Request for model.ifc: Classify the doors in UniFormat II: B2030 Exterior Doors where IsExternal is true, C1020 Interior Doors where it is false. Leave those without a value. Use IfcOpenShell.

First a look at what the model holds.

```python
import ifcopenshell
import ifcopenshell.util.element

model = ifcopenshell.open("model.ifc")
print(model.schema)
print("classifications:", [c.Name for c in model.by_type("IfcClassification")])
values = [ifcopenshell.util.element.get_pset(e, "Pset_DoorCommon", "IsExternal") for e in model.by_type("IfcDoor")]
for value in (True, False, None):
    print("IsExternal", value, values.count(value))
```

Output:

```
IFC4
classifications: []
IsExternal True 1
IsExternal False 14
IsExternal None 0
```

```python
import ifcopenshell
import ifcopenshell.api.classification
import ifcopenshell.util.element

model = ifcopenshell.open("model.ifc")

system = ifcopenshell.api.classification.add_classification(model, classification="UniFormat II")

doors = model.by_type("IfcDoor")
external = {e: ifcopenshell.util.element.get_pset(e, "Pset_DoorCommon", "IsExternal") for e in doors}
for flag, code, name in ((True, "B2030", "Exterior Doors"), (False, "C1020", "Interior Doors")):
    products = [e for e in doors if external[e] is flag]
    ifcopenshell.api.classification.add_reference(
        model, products=products, classification=system, identification=code, name=name
    )
    print(code, len(products))

model.write("model_v2.ifc")
```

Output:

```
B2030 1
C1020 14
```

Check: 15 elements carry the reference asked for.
